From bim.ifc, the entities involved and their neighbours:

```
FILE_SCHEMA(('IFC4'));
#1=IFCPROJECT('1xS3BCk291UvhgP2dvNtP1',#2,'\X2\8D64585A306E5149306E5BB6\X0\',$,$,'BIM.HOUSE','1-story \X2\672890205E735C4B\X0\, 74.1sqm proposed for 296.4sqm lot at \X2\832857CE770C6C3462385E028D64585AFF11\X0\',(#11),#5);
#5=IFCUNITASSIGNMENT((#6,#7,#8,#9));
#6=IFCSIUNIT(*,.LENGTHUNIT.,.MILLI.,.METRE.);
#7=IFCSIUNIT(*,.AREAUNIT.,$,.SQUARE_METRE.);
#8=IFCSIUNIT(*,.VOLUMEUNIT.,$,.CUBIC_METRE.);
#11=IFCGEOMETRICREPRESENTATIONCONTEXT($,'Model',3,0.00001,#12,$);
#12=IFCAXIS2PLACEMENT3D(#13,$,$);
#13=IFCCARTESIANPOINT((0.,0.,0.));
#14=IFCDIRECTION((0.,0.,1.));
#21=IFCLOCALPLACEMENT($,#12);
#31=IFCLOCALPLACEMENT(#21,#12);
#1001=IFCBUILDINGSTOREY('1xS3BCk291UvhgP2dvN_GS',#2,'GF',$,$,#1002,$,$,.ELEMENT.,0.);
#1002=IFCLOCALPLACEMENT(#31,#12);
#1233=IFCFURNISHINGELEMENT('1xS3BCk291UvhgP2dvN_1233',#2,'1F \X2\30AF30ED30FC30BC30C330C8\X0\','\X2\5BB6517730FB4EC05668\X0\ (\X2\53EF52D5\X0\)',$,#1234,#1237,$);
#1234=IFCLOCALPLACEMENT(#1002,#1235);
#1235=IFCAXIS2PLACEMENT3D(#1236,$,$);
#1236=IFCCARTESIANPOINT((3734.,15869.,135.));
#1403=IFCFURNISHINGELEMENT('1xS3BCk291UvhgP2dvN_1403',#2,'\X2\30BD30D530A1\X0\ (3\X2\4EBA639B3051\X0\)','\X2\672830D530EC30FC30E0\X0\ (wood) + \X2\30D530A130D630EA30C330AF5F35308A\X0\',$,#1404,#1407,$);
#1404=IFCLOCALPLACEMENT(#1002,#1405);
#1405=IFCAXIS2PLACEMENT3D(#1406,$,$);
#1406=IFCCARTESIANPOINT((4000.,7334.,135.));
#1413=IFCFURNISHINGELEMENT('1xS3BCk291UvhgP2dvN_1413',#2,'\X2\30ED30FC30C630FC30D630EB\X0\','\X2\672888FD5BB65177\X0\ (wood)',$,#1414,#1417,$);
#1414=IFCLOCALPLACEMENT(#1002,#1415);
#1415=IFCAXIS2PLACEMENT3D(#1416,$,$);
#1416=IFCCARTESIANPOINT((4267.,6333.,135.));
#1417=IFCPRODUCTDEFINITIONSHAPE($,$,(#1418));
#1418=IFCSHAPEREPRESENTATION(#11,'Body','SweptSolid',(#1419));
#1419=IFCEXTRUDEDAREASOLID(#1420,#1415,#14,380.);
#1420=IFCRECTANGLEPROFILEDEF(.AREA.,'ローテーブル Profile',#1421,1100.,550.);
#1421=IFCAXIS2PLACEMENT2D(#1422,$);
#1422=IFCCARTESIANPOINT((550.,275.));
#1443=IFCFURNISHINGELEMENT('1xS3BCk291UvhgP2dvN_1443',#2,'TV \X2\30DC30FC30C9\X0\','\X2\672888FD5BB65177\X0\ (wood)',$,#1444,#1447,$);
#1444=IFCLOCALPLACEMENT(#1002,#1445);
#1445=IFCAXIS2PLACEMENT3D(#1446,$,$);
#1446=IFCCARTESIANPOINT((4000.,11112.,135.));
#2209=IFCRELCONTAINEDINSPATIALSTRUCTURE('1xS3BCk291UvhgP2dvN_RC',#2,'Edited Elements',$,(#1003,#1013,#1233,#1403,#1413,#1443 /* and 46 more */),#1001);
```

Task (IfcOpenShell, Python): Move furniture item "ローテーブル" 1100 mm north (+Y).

```python
import ifcopenshell
import ifcopenshell.api.geometry
import ifcopenshell.util.placement
import ifcopenshell.util.unit

model = ifcopenshell.open("bim.ifc")
unit_scale = ifcopenshell.util.unit.calculate_unit_scale(model)

item = model.by_guid("1xS3BCk291UvhgP2dvN_1413")
matrix = ifcopenshell.util.placement.get_local_placement(item.ObjectPlacement)
matrix[1, 3] += 1.1 / unit_scale
ifcopenshell.api.geometry.edit_object_placement(model, product=item, matrix=matrix, is_si=False)

print(ifcopenshell.util.placement.get_local_placement(item.ObjectPlacement).round(3) + 0.0)

model.write("bim-out.ifc")
```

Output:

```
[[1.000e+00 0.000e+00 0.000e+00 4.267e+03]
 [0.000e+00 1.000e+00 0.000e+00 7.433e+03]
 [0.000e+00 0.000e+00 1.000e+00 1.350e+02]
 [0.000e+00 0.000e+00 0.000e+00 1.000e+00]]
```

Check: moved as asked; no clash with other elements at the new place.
